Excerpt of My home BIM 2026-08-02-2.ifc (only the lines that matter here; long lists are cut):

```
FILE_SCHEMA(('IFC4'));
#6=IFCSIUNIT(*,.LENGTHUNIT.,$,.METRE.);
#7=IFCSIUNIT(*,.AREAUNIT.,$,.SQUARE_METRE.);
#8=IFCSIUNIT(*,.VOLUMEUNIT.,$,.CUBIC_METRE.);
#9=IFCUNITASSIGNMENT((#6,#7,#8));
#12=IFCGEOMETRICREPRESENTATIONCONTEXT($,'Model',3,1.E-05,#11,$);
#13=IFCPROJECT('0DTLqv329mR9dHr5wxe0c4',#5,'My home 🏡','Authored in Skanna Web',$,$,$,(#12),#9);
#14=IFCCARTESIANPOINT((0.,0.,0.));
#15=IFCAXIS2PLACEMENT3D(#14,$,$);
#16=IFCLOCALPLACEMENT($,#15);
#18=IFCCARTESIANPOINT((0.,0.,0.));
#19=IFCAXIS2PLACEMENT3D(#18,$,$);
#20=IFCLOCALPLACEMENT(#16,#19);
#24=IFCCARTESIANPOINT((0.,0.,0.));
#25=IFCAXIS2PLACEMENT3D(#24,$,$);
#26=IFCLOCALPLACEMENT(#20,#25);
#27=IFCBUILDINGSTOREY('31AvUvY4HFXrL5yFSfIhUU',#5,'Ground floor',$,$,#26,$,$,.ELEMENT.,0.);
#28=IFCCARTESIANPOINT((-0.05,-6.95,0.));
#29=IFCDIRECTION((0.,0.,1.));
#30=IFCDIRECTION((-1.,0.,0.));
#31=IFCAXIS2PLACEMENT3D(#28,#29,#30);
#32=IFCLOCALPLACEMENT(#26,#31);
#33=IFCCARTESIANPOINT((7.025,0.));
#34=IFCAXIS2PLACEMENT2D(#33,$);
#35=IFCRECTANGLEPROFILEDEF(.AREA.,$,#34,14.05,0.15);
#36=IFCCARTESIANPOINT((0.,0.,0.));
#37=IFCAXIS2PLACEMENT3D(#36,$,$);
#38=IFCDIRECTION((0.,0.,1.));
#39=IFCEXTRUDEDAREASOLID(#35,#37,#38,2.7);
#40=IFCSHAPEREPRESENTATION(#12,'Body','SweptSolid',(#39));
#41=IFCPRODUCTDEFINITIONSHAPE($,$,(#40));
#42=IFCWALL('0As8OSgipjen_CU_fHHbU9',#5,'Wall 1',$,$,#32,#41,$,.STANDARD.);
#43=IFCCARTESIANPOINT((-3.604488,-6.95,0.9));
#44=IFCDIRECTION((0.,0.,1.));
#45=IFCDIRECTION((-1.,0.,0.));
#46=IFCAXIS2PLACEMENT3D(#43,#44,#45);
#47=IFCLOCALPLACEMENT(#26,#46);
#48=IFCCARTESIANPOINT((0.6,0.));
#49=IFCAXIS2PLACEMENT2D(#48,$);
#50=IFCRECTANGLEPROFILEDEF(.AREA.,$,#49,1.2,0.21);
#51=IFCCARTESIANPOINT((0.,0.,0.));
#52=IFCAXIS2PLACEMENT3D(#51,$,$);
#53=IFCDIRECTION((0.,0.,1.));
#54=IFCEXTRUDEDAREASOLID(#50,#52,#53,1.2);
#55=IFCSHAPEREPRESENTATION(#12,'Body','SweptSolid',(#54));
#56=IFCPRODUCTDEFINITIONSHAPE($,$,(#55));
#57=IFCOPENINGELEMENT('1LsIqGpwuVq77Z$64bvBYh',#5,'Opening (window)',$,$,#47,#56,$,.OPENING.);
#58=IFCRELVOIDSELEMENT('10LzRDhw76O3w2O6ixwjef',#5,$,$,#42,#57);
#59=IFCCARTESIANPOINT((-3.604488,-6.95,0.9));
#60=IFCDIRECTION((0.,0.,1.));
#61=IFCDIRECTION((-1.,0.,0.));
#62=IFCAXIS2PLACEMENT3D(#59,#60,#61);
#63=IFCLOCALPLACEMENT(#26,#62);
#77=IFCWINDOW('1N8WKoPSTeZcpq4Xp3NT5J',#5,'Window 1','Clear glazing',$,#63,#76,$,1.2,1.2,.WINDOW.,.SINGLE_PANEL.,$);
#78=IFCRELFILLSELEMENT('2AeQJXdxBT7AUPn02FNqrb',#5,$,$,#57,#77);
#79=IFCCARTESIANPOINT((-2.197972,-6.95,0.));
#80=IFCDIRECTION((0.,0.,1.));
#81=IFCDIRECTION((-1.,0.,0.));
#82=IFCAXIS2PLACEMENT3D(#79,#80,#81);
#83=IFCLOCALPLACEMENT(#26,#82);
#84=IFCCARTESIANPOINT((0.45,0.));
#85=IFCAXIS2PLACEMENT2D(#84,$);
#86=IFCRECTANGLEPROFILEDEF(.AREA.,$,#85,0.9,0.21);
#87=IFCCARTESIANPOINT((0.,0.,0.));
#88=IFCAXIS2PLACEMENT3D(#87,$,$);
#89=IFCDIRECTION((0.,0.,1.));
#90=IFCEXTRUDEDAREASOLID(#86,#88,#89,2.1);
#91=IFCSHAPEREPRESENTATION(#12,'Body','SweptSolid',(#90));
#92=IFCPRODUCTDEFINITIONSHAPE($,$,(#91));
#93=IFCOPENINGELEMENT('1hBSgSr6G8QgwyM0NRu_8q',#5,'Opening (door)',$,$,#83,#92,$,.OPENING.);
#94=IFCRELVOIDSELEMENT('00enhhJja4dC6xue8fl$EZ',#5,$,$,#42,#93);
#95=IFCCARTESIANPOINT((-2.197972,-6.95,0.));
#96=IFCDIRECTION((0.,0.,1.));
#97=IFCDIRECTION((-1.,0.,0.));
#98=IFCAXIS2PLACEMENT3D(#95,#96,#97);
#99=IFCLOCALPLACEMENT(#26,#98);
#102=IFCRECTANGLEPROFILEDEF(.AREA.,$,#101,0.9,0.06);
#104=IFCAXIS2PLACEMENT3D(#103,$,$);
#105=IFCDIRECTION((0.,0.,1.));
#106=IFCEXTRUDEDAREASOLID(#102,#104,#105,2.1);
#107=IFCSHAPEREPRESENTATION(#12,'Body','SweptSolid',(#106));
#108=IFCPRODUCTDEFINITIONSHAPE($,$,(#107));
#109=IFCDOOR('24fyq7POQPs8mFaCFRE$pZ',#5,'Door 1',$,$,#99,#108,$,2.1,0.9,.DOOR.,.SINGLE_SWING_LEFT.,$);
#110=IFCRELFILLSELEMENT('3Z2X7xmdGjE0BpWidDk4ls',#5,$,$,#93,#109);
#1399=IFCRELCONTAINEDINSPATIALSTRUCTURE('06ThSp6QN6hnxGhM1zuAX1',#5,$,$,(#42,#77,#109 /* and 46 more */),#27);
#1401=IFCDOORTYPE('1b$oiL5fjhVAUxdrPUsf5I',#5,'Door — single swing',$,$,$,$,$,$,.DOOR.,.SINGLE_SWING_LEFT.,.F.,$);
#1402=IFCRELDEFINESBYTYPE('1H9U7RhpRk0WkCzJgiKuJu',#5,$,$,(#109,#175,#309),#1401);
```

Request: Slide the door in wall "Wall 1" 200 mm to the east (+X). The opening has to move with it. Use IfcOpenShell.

```python
import ifcopenshell
import ifcopenshell.api.geometry
import ifcopenshell.util.placement

model = ifcopenshell.open("My home BIM 2026-08-02-2.ifc")

door = model.by_guid("24fyq7POQPs8mFaCFRE$pZ")
opening = door.FillsVoids[0].RelatingOpeningElement
wall = opening.VoidsElements[0].RelatingBuildingElement

wall_matrix = ifcopenshell.util.placement.get_local_placement(wall.ObjectPlacement)
shift = wall_matrix[:3, 0] * -0.2
before = ifcopenshell.util.placement.get_local_placement(door.ObjectPlacement)[:3, 3].copy()

# The door is not placed relative to its opening, so move both.
for product in (opening, door):
    matrix = ifcopenshell.util.placement.get_local_placement(product.ObjectPlacement)
    matrix[:3, 3] += shift
    ifcopenshell.api.geometry.edit_object_placement(model, product=product, matrix=matrix, is_si=False)

after = ifcopenshell.util.placement.get_local_placement(door.ObjectPlacement)[:3, 3]
print("door moved by", (after - before).round(3) + 0.0)

model.write("My home BIM 2026-08-02-2_v2.ifc")
```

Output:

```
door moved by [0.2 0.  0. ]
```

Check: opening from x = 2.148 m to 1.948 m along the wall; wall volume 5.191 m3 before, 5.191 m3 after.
